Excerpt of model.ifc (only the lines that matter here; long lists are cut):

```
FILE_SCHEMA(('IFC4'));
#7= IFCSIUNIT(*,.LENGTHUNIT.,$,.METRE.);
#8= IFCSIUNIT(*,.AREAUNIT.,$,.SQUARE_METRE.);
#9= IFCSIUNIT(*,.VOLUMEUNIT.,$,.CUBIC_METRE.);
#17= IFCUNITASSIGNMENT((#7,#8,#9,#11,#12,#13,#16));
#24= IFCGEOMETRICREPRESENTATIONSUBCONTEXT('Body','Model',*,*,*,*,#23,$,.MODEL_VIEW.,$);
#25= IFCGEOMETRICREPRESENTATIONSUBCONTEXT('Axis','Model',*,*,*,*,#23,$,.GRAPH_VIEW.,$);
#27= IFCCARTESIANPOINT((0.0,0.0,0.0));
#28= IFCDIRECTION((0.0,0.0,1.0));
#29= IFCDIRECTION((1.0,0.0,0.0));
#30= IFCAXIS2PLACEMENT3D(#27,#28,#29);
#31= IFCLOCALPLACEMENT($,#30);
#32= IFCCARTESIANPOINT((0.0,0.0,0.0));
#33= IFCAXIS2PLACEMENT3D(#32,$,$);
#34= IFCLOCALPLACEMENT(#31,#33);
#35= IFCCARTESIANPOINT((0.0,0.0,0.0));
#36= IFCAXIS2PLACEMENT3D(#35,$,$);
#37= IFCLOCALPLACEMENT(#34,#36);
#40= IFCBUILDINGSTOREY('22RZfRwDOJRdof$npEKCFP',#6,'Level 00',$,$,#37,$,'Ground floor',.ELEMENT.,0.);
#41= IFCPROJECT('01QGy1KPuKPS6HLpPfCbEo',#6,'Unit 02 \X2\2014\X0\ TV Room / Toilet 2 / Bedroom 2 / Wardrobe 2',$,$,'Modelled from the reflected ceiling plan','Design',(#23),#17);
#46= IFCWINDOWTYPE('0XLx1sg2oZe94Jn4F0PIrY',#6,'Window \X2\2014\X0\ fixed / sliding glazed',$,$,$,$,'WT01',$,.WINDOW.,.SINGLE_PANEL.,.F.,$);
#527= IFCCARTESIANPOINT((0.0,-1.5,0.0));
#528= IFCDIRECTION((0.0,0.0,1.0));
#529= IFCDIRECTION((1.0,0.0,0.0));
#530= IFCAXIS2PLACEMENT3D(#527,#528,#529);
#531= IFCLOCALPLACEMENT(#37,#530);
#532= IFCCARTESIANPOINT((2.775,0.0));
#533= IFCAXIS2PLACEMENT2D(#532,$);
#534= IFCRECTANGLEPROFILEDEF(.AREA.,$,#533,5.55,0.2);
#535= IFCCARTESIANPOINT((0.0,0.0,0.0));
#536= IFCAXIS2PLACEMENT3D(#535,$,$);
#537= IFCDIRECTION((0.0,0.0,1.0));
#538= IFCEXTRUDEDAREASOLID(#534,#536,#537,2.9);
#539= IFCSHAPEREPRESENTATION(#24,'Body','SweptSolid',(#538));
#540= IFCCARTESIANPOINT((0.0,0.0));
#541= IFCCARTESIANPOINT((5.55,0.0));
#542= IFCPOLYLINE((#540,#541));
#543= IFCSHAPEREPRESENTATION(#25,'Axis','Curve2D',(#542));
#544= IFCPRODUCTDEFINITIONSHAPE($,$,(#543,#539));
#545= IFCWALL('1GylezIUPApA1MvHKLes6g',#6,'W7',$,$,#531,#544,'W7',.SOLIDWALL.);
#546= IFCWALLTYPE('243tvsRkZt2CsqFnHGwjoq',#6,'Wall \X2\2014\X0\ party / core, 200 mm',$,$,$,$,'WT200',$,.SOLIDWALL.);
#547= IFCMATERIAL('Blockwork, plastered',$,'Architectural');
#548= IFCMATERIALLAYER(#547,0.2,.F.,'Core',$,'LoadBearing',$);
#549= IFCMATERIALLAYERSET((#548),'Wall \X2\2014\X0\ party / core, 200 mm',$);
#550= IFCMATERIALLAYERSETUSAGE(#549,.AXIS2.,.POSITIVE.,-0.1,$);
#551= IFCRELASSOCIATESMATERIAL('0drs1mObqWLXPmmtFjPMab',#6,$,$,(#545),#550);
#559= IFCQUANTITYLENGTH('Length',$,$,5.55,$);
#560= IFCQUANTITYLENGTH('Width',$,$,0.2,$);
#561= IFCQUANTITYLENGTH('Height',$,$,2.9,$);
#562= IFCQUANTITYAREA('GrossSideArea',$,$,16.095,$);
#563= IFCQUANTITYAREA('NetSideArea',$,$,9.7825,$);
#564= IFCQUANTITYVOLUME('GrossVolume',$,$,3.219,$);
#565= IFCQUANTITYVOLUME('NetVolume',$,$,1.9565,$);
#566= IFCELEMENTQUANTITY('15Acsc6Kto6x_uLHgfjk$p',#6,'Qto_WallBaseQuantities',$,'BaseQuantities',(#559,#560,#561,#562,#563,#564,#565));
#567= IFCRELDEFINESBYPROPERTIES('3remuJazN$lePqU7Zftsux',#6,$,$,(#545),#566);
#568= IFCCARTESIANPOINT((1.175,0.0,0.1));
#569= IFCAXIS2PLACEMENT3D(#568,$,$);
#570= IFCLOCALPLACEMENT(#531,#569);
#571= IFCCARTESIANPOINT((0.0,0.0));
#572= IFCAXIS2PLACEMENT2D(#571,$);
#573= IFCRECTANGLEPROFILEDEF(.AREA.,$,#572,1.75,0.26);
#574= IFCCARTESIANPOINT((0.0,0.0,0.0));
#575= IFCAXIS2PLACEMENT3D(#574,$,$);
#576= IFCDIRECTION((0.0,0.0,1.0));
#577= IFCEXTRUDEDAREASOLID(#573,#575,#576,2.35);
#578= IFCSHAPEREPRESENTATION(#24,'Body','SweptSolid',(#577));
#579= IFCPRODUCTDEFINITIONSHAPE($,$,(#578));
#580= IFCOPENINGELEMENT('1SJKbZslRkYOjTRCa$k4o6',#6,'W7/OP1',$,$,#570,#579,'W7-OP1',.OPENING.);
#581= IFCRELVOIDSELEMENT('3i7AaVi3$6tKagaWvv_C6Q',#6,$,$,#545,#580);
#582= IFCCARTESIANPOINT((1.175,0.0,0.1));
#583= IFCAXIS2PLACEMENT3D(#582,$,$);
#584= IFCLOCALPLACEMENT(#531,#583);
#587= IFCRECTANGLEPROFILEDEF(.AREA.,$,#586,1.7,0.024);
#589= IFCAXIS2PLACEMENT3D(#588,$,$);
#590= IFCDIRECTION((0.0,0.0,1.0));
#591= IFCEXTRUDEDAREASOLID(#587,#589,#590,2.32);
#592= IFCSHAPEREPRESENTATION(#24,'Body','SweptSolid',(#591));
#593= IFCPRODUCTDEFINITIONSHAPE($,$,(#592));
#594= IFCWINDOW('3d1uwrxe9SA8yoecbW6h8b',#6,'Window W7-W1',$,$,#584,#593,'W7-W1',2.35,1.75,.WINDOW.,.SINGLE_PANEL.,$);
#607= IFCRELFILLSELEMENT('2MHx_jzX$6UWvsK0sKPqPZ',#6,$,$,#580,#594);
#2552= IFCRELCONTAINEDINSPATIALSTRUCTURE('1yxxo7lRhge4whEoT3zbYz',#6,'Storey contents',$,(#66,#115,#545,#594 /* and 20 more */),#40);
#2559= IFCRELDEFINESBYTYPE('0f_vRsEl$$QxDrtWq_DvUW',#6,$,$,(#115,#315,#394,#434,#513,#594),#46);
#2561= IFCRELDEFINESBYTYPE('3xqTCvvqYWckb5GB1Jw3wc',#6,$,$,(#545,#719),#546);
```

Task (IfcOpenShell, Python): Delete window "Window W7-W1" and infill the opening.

```python
import ifcopenshell
import ifcopenshell.api.feature
import ifcopenshell.api.pset
import ifcopenshell.api.root
import ifcopenshell.geom
import ifcopenshell.util.element
import ifcopenshell.util.shape
import ifcopenshell.util.unit

model = ifcopenshell.open("model.ifc")
area_scale = ifcopenshell.util.unit.calculate_unit_scale(model, "AREAUNIT")
volume_scale = ifcopenshell.util.unit.calculate_unit_scale(model, "VOLUMEUNIT")
settings = ifcopenshell.geom.settings()


def volume(element):
    """Net volume in cubic metres, openings subtracted."""
    shape = ifcopenshell.geom.create_shape(settings, element)
    return ifcopenshell.util.shape.get_volume(shape.geometry)


window = model.by_guid("3d1uwrxe9SA8yoecbW6h8b")
opening = window.FillsVoids[0].RelatingOpeningElement
wall = opening.VoidsElements[0].RelatingBuildingElement
before = volume(wall)

ifcopenshell.api.root.remove_product(model, product=window)
ifcopenshell.api.feature.remove_feature(model, feature=opening)

after = volume(wall)
thickness = 0.2  # wall thickness in metres

# Update the wall's stored quantities.
qto = model.by_id(ifcopenshell.util.element.get_pset(wall, "Qto_WallBaseQuantities", should_inherit=False)["id"])
ifcopenshell.api.pset.edit_qto(model, qto=qto, properties={
    "NetSideArea": after / thickness / area_scale,
    "NetVolume": after / volume_scale,
})

print(f"wall volume {before:.3f} -> {after:.3f} m3")

model.write("model_rev.ifc")
```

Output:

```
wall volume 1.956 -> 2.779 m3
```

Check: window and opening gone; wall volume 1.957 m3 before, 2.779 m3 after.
